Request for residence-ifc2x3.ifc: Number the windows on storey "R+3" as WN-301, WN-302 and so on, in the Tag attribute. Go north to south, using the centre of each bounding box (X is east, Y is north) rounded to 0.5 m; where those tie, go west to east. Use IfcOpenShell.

First a look at what the model holds.

```python
import ifcopenshell
import ifcopenshell.util.element
import ifcopenshell.util.placement

model = ifcopenshell.open("residence-ifc2x3.ifc")
print(model.schema)
storey = next(s for s in model.by_type("IfcBuildingStorey") if s.Name == "R+3")
windows = [e for e in ifcopenshell.util.element.get_decomposition(storey) if e.is_a("IfcWindow")]
for e in sorted(windows, key=lambda e: e.id()):
    origin = ifcopenshell.util.placement.get_local_placement(e.ObjectPlacement)[:3, 3]
    print(e.id(), e.Tag, e.Name, origin.round(2) + 0.0, sep=" | ")
```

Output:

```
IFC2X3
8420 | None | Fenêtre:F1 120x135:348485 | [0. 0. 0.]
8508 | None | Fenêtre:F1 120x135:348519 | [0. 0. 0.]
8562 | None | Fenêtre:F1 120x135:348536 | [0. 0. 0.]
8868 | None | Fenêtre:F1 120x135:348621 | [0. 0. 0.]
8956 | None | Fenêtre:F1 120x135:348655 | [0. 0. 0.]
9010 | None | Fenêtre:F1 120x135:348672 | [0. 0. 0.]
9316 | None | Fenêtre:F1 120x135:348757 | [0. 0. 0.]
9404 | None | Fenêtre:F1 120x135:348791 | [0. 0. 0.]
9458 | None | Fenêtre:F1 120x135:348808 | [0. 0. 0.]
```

```python
import ifcopenshell
import ifcopenshell.geom
import ifcopenshell.util.element
import ifcopenshell.util.shape

model = ifcopenshell.open("residence-ifc2x3.ifc")
settings = ifcopenshell.geom.settings()
settings.set("use-world-coords", True)


def centre(element):
    shape = ifcopenshell.geom.create_shape(settings, element)
    return ifcopenshell.util.shape.get_bbox_centroid(shape.geometry)


storey = next(s for s in model.by_type("IfcBuildingStorey") if s.Name == "R+3")
windows = [e for e in ifcopenshell.util.element.get_decomposition(storey) if e.is_a("IfcWindow")]

# Insertion points can sit at a corner or the storey origin, so sort by the geometry (in metres).
centres = {e: centre(e) for e in windows}
windows.sort(key=lambda e: (-round(centres[e][1] / 0.5), centres[e][0]))

for i, e in enumerate(windows, start=1):
    number = f"WN-3{i:02d}"
    e.Tag = number
    print(e.id(), number)

model.write("residence-ifc2x3_v2.ifc")
```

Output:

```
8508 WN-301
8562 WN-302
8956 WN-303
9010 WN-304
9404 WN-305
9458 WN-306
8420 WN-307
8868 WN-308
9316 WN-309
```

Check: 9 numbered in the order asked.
